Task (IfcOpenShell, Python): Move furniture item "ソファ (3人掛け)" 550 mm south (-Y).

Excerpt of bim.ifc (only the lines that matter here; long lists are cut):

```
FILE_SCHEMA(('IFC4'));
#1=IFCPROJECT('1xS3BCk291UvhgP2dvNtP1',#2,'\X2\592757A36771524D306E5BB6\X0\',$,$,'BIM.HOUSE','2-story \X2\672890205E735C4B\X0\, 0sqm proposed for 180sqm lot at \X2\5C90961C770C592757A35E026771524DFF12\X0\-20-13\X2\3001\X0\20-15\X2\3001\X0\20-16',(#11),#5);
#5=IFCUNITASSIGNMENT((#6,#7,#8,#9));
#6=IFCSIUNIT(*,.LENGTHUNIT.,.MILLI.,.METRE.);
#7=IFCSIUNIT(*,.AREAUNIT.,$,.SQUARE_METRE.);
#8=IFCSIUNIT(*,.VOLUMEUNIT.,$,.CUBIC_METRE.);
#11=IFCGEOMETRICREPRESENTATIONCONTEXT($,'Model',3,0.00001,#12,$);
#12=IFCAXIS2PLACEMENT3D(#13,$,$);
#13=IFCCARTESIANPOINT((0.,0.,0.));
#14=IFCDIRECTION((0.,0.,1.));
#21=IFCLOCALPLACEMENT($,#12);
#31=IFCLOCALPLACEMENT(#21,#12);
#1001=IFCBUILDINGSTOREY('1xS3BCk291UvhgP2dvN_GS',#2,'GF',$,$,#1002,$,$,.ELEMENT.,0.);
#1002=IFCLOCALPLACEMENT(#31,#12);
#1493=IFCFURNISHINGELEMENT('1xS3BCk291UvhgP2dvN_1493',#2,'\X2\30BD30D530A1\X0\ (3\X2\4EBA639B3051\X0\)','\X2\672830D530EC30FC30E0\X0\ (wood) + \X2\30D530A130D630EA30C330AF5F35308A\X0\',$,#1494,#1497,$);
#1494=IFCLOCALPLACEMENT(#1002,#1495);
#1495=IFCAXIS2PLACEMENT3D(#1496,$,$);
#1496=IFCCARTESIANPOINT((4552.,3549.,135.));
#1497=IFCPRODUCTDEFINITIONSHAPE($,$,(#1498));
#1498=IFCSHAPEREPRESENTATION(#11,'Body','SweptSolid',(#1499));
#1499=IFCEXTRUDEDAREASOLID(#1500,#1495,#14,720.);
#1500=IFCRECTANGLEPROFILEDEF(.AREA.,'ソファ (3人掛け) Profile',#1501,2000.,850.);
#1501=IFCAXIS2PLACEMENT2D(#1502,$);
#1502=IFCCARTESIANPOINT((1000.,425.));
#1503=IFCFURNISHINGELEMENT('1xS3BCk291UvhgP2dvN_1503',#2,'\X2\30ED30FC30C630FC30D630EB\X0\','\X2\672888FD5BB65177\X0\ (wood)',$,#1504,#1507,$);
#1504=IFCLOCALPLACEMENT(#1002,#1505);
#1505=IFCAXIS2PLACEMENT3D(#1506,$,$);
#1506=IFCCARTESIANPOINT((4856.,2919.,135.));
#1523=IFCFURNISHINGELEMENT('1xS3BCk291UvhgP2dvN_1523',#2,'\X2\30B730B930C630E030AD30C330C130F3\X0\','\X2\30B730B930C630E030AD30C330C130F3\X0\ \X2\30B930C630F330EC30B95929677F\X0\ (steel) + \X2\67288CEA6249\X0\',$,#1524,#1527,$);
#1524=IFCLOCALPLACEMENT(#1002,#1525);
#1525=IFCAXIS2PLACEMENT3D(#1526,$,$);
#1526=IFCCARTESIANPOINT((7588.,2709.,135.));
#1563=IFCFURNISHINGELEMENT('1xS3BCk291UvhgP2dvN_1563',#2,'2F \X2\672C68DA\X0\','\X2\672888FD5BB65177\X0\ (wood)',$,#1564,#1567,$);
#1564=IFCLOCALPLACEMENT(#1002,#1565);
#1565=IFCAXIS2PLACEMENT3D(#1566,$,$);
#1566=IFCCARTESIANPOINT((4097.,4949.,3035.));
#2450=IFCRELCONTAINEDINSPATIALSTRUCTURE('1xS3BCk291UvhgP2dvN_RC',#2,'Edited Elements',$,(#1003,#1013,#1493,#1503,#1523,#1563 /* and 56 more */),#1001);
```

```python
import ifcopenshell
import ifcopenshell.api.geometry
import ifcopenshell.util.placement

model = ifcopenshell.open("bim.ifc")

item = model.by_guid("1xS3BCk291UvhgP2dvN_1493")
matrix = ifcopenshell.util.placement.get_local_placement(item.ObjectPlacement)
matrix[1, 3] -= 550.0
ifcopenshell.api.geometry.edit_object_placement(model, product=item, matrix=matrix, is_si=False)

print(ifcopenshell.util.placement.get_local_placement(item.ObjectPlacement).round(3) + 0.0)

model.write("bim_rev.ifc")
```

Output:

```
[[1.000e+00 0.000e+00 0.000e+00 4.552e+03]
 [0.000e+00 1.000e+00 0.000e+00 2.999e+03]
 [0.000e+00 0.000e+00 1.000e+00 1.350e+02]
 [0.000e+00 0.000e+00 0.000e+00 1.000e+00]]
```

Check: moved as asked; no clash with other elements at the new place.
